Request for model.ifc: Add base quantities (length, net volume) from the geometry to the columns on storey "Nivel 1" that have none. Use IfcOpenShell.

First a look at what the model holds.

```python
import ifcopenshell
import ifcopenshell.util.element
import ifcopenshell.util.unit

model = ifcopenshell.open("model.ifc")
print(model.schema)
for unit_type in ("LENGTHUNIT", "AREAUNIT", "VOLUMEUNIT"):
    print(unit_type, ifcopenshell.util.unit.calculate_unit_scale(model, unit_type))
storey = next(s for s in model.by_type("IfcBuildingStorey") if s.Name == "Nivel 1")
columns = [e for e in ifcopenshell.util.element.get_decomposition(storey) if e.is_a("IfcColumn")]
for e in sorted(columns, key=lambda e: e.id()):
    print(e.id(), e.is_a(), e.Name, list(ifcopenshell.util.element.get_psets(e, qtos_only=True)), sep=" | ")
```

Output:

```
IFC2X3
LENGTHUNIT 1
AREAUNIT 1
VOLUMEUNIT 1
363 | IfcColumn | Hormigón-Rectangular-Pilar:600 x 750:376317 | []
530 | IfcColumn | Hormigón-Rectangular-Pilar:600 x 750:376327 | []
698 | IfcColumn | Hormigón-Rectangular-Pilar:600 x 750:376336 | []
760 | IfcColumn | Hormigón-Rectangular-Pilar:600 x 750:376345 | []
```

```python
import ifcopenshell
import ifcopenshell.api.pset
import ifcopenshell.geom
import ifcopenshell.util.element
import ifcopenshell.util.shape
import ifcopenshell.util.unit

model = ifcopenshell.open("model.ifc")
unit_scale = ifcopenshell.util.unit.calculate_unit_scale(model)
volume_scale = ifcopenshell.util.unit.calculate_unit_scale(model, "VOLUMEUNIT")
settings = ifcopenshell.geom.settings()

storey = next(s for s in model.by_type("IfcBuildingStorey") if s.Name == "Nivel 1")
columns = [e for e in ifcopenshell.util.element.get_decomposition(storey) if e.is_a("IfcColumn")]

for e in sorted(columns, key=lambda e: e.id()):
    if ifcopenshell.util.element.get_psets(e, qtos_only=True, should_inherit=False):
        continue
    # Geometry comes back in metres, in the element's own axes.
    shape = ifcopenshell.geom.create_shape(settings, e)
    values = {
        "Length": ifcopenshell.util.shape.get_z(shape.geometry) / unit_scale,
        "NetVolume": ifcopenshell.util.shape.get_volume(shape.geometry) / volume_scale,
    }
    qto = ifcopenshell.api.pset.add_qto(model, product=e, name="BaseQuantities")
    ifcopenshell.api.pset.edit_qto(model, qto=qto, properties=values)
    print(e.id(), {k: round(v, 3) for k, v in values.items()})

model.write("model-out.ifc")
```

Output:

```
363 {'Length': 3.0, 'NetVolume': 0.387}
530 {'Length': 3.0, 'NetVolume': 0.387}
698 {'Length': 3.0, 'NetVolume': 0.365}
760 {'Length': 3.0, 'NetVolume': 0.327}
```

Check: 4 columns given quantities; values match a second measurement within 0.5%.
